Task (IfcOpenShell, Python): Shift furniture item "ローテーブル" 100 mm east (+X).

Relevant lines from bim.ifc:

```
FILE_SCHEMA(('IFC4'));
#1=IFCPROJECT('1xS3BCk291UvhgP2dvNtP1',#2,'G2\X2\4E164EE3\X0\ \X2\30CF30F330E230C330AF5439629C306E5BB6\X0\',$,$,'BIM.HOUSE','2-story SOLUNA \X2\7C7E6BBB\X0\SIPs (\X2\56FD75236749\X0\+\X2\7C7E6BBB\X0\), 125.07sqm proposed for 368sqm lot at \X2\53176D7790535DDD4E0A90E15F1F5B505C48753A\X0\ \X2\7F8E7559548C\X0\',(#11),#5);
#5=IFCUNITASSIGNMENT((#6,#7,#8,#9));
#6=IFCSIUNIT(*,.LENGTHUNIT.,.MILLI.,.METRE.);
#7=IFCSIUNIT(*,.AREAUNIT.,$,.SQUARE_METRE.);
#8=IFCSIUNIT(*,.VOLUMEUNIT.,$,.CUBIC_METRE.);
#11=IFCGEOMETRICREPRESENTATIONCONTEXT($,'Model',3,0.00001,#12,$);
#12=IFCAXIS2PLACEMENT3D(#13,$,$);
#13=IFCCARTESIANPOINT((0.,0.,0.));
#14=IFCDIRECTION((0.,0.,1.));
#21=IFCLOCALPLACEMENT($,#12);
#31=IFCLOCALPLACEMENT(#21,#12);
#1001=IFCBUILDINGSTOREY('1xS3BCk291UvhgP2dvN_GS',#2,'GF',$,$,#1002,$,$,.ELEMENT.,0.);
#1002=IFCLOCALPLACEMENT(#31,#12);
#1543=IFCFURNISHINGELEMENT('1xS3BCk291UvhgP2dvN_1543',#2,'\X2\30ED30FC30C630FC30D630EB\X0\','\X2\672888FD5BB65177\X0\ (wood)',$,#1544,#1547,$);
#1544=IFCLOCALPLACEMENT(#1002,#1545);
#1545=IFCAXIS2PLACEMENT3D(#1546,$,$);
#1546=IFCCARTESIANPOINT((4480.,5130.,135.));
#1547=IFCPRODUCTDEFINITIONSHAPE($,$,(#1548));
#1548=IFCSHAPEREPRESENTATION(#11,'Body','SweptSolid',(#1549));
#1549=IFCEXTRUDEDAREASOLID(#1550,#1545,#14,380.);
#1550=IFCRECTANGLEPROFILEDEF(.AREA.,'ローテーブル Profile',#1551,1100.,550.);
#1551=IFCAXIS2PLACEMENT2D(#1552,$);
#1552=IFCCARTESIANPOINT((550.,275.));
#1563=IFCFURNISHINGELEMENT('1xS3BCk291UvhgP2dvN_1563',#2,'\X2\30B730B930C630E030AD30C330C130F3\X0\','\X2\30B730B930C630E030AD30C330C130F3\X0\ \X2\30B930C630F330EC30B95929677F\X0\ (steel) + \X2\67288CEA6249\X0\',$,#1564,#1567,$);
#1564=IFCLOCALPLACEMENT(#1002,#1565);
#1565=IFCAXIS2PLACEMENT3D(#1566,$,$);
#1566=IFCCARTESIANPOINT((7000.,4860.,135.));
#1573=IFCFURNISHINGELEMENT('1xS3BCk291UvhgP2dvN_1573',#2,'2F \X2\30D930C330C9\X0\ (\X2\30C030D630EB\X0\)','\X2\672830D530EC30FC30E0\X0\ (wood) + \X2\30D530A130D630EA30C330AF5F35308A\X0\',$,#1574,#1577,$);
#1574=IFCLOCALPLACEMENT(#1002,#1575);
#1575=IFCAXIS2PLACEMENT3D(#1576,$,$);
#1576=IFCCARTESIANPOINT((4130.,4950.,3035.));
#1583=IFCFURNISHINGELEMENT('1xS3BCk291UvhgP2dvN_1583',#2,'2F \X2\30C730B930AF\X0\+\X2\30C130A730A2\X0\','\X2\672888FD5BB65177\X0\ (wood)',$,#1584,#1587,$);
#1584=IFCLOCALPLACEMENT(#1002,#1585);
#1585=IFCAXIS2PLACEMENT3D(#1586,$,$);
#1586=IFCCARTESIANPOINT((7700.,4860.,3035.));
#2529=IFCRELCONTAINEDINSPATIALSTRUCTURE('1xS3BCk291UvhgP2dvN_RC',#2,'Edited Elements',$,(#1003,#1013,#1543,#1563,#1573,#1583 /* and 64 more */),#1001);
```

```python
import ifcopenshell
import ifcopenshell.api.geometry
import ifcopenshell.util.placement
import ifcopenshell.util.unit

model = ifcopenshell.open("bim.ifc")
unit_scale = ifcopenshell.util.unit.calculate_unit_scale(model)

item = model.by_guid("1xS3BCk291UvhgP2dvN_1543")
matrix = ifcopenshell.util.placement.get_local_placement(item.ObjectPlacement)
matrix[0, 3] += 0.1 / unit_scale
ifcopenshell.api.geometry.edit_object_placement(model, product=item, matrix=matrix, is_si=False)

print(ifcopenshell.util.placement.get_local_placement(item.ObjectPlacement).round(3) + 0.0)

model.write("bim_edited.ifc")
```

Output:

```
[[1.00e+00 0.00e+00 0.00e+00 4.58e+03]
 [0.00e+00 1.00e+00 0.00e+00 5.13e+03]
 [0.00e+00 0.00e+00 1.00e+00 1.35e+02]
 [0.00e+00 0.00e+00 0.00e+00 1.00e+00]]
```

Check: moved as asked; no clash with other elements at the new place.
